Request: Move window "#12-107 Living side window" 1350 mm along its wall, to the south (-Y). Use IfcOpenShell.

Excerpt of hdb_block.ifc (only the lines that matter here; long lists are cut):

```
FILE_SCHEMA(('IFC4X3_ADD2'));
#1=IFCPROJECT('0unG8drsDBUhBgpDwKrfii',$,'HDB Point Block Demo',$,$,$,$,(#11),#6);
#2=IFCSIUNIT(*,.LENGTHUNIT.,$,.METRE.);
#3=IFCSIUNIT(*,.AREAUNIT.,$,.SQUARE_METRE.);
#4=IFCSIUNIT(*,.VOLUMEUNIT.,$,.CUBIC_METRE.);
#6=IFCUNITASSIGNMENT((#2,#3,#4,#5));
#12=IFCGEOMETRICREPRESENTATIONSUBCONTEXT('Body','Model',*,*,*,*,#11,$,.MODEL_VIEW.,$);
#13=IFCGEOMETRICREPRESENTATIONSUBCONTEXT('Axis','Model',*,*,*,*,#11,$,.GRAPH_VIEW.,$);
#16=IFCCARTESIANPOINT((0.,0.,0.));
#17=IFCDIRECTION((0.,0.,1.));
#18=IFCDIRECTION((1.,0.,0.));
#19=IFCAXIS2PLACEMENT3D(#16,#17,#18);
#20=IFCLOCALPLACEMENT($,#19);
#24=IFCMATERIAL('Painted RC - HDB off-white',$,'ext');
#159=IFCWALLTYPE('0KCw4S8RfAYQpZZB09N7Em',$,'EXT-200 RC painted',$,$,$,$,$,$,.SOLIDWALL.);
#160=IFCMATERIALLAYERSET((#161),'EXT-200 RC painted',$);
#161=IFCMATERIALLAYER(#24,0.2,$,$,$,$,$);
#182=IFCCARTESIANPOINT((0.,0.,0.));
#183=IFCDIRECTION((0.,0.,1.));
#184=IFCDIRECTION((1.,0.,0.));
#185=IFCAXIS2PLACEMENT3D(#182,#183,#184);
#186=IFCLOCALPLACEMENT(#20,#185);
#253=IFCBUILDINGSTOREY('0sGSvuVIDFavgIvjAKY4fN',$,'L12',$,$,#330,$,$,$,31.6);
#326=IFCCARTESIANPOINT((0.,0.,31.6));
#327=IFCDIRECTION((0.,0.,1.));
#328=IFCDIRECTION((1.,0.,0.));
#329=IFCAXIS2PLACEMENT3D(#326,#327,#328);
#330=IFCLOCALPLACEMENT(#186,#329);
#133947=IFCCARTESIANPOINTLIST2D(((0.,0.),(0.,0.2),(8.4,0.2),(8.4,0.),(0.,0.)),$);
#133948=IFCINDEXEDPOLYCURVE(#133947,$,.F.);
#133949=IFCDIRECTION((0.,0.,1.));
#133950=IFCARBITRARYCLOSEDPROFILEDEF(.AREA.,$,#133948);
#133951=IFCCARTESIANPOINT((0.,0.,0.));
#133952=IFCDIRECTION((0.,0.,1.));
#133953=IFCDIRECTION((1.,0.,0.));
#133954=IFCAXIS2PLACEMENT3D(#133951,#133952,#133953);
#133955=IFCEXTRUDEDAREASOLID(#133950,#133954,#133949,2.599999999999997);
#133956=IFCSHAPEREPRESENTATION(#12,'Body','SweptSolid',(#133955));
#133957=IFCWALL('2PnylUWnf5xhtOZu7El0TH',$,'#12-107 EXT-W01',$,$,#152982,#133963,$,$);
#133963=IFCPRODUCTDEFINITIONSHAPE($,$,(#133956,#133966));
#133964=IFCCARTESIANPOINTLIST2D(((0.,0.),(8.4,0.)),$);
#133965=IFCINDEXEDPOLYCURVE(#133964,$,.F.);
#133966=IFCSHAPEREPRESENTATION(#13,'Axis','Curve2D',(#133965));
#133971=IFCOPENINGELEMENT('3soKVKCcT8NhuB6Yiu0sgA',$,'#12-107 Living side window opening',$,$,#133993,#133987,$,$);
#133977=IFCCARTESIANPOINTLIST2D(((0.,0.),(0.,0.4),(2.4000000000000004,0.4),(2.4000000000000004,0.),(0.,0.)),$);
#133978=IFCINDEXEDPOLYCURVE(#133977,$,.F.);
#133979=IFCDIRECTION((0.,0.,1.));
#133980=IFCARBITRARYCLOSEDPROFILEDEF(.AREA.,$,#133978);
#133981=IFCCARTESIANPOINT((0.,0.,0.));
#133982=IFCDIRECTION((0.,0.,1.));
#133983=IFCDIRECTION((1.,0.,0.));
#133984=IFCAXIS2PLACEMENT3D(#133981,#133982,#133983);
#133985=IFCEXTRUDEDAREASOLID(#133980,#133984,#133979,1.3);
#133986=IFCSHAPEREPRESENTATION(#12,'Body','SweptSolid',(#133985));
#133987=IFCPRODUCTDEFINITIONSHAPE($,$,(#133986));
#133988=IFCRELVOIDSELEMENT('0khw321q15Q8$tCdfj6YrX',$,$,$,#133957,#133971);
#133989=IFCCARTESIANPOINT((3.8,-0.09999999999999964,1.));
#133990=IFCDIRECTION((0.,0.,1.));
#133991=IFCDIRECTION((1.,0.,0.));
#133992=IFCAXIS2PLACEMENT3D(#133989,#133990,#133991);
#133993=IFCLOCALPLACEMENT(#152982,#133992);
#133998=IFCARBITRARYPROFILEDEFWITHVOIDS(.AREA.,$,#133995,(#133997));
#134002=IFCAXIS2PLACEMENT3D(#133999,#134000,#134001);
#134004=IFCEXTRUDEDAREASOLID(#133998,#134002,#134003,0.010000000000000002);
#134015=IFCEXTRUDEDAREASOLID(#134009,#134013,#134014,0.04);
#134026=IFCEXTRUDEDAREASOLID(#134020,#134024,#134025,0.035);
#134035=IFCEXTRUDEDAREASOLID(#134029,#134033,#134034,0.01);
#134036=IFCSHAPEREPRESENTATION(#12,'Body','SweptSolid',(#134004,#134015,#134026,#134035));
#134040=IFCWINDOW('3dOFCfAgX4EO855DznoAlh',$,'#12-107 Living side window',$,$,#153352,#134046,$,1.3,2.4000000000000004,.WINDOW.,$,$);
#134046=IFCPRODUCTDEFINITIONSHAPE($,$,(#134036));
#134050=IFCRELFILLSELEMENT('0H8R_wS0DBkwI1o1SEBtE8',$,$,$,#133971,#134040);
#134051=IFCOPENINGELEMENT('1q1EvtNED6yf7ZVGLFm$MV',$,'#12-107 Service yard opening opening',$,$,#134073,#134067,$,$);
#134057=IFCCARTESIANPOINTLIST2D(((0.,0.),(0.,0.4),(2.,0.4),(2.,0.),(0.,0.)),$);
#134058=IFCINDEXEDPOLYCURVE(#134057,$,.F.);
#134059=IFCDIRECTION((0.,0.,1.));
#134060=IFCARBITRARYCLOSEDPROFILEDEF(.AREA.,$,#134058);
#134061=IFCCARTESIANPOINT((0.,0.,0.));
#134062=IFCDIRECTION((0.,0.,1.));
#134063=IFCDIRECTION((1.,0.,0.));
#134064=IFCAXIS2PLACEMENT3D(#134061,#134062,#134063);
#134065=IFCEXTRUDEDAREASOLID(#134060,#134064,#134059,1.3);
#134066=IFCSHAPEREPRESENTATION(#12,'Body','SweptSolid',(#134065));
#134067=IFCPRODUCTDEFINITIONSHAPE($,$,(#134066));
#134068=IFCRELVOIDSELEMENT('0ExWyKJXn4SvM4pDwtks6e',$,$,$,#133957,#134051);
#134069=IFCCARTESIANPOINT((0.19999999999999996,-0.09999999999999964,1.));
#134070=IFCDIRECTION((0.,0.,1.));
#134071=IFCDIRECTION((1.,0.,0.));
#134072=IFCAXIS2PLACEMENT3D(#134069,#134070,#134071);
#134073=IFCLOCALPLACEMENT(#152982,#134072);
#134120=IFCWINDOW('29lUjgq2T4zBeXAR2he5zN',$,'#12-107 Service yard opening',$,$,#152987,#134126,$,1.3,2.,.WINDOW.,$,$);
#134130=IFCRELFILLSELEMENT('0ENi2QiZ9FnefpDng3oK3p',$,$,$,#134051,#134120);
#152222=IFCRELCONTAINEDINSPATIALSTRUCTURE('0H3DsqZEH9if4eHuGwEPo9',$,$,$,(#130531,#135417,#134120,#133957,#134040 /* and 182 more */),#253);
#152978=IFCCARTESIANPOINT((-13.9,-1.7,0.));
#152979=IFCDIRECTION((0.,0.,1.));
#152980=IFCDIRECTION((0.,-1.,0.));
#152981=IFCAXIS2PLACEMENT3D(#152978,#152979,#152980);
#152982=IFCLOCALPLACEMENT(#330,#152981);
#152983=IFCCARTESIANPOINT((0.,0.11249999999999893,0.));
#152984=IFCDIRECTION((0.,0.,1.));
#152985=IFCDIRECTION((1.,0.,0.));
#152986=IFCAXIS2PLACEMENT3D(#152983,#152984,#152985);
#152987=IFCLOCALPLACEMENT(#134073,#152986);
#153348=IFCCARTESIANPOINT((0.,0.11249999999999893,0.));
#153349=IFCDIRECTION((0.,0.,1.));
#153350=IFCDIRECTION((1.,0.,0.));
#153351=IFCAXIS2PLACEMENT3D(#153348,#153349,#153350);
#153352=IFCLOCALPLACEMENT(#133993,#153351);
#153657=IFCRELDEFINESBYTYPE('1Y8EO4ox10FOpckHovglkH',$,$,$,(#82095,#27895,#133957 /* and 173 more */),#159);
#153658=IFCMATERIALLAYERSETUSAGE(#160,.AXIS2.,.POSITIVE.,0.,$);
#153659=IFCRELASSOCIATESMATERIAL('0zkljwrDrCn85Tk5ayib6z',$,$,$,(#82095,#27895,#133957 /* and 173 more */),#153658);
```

```python
import ifcopenshell
import ifcopenshell.api.geometry
import ifcopenshell.util.placement
import ifcopenshell.util.unit

model = ifcopenshell.open("hdb_block.ifc")
unit_scale = ifcopenshell.util.unit.calculate_unit_scale(model)

window = model.by_id(134040)
opening = window.FillsVoids[0].RelatingOpeningElement
wall = opening.VoidsElements[0].RelatingBuildingElement

wall_matrix = ifcopenshell.util.placement.get_local_placement(wall.ObjectPlacement)
shift = wall_matrix[:3, 0] * 1.35 / unit_scale
before = ifcopenshell.util.placement.get_local_placement(window.ObjectPlacement)[:3, 3].copy()

# The window is placed relative to its opening, so it follows when the opening moves.
matrix = ifcopenshell.util.placement.get_local_placement(opening.ObjectPlacement)
matrix[:3, 3] += shift
ifcopenshell.api.geometry.edit_object_placement(
    model, product=opening, matrix=matrix, is_si=False, should_transform_children=True
)

after = ifcopenshell.util.placement.get_local_placement(window.ObjectPlacement)[:3, 3]
print("window moved by", (after - before).round(3) + 0.0)

model.write("hdb_block-out.ifc")
```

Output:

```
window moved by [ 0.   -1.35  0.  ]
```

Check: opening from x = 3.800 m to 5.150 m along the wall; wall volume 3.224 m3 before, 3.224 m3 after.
